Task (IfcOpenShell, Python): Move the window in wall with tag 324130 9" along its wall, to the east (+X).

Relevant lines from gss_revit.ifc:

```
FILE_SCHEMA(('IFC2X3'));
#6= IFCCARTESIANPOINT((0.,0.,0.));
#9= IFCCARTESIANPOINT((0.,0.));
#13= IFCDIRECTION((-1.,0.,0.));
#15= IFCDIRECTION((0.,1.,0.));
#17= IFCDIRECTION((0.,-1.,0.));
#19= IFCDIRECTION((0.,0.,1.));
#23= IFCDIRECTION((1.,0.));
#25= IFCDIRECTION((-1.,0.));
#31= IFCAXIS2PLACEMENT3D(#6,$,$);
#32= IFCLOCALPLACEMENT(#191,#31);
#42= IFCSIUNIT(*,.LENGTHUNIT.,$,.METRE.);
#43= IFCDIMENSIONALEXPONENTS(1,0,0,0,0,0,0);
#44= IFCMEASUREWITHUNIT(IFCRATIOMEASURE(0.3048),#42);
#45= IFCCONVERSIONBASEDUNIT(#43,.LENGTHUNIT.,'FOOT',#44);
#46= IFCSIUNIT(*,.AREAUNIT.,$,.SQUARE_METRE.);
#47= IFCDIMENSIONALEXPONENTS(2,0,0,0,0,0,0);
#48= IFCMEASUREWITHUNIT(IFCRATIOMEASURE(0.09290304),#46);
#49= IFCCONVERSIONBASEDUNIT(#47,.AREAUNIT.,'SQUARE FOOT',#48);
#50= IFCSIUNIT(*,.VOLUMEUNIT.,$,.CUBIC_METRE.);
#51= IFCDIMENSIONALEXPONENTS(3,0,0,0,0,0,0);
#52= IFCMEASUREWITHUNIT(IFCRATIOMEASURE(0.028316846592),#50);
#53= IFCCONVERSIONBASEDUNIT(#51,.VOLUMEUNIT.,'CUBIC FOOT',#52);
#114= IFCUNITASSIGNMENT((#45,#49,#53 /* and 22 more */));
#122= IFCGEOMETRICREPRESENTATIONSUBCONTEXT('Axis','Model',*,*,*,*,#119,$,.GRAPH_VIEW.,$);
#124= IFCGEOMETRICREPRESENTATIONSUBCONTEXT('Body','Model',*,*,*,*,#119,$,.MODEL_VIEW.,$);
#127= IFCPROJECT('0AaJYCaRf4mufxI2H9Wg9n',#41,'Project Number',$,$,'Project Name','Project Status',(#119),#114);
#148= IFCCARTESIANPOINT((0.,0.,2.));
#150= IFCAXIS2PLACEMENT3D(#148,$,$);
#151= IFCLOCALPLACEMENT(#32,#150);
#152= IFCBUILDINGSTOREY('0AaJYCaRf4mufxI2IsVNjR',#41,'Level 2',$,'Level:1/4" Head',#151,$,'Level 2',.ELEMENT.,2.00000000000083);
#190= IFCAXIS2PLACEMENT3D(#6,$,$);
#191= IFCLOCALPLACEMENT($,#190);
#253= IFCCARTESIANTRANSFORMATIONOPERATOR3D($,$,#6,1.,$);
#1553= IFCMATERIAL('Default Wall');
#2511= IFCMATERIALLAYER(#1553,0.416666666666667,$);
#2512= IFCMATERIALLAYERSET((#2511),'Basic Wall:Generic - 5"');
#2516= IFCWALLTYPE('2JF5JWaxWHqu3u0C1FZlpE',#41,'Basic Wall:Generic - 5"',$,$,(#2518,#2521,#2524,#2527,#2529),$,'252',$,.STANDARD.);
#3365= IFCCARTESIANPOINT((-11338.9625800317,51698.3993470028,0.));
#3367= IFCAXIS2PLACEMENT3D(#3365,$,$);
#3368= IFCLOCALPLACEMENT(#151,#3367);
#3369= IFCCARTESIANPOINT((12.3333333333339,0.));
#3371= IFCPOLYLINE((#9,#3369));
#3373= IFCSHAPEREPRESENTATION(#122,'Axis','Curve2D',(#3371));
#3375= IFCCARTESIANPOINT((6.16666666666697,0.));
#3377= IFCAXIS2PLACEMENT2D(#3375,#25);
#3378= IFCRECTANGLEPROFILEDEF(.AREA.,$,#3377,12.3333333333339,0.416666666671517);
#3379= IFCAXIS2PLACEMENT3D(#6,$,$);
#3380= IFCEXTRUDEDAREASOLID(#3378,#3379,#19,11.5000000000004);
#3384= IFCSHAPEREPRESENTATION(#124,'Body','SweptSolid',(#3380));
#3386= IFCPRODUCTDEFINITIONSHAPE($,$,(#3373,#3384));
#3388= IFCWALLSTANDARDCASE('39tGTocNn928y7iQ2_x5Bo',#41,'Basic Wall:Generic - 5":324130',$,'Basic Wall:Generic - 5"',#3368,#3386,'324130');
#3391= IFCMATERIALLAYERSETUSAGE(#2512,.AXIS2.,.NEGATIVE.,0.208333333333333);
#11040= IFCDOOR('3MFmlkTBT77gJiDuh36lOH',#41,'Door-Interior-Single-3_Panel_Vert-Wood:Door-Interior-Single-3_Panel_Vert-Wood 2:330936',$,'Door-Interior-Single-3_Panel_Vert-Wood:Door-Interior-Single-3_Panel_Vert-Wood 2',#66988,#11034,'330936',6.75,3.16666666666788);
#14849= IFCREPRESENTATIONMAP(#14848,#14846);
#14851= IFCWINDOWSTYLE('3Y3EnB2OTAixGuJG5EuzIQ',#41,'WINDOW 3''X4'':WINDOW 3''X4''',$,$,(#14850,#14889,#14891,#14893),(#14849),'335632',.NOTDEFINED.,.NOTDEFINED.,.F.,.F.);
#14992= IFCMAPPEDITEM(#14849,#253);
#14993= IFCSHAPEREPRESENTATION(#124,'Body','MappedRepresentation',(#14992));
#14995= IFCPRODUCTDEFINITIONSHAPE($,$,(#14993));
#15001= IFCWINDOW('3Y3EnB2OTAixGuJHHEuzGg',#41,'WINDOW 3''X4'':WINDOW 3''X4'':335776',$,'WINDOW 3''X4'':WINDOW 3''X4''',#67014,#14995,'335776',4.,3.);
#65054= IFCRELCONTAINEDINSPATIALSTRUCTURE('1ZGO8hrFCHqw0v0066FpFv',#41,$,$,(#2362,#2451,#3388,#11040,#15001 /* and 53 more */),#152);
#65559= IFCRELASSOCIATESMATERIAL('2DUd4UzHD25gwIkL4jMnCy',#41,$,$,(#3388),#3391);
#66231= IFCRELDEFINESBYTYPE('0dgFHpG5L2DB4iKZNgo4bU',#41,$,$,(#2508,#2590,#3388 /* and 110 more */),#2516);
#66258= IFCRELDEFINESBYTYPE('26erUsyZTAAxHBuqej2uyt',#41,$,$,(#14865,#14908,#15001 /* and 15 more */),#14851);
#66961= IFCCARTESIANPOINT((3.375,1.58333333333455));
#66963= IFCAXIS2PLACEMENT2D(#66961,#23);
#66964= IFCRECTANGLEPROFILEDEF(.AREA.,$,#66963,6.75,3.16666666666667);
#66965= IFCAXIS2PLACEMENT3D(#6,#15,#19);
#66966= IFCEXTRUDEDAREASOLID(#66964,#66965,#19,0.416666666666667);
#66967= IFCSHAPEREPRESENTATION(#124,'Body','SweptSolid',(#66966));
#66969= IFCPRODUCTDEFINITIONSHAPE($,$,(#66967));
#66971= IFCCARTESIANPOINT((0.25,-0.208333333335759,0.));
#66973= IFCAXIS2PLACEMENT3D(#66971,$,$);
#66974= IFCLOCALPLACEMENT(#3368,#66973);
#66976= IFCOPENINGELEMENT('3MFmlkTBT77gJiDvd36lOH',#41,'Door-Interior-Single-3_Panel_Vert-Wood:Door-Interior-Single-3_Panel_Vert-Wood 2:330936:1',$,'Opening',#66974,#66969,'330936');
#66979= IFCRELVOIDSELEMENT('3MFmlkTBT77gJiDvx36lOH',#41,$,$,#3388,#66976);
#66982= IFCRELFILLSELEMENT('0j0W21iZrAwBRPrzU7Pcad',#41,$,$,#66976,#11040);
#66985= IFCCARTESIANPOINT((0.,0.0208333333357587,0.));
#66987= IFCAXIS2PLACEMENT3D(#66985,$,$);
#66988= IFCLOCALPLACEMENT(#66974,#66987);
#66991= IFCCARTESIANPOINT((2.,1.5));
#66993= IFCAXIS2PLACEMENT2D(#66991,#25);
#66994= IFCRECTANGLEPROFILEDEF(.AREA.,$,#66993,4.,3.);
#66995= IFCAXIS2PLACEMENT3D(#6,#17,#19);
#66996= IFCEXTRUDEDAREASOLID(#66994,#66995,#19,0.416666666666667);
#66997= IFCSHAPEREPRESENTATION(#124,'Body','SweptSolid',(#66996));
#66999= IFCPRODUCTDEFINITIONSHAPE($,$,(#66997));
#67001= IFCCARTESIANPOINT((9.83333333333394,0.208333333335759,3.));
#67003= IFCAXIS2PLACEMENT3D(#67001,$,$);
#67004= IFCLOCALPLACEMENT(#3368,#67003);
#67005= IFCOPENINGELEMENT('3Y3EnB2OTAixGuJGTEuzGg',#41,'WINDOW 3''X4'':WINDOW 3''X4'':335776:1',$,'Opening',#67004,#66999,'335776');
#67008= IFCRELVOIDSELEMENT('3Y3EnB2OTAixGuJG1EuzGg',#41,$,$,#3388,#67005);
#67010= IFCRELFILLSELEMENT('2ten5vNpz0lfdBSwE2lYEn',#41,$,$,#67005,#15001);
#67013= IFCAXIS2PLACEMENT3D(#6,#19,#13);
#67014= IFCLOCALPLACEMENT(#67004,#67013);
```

```python
import ifcopenshell
import ifcopenshell.api.geometry
import ifcopenshell.util.placement
import ifcopenshell.util.unit

model = ifcopenshell.open("gss_revit.ifc")
unit_scale = ifcopenshell.util.unit.calculate_unit_scale(model)

window = model.by_guid("3Y3EnB2OTAixGuJHHEuzGg")
opening = window.FillsVoids[0].RelatingOpeningElement
wall = opening.VoidsElements[0].RelatingBuildingElement

wall_matrix = ifcopenshell.util.placement.get_local_placement(wall.ObjectPlacement)
shift = wall_matrix[:3, 0] * 9 * 0.0254 / unit_scale
before = ifcopenshell.util.placement.get_local_placement(window.ObjectPlacement)[:3, 3].copy()

# The window is placed relative to its opening, so it follows when the opening moves.
matrix = ifcopenshell.util.placement.get_local_placement(opening.ObjectPlacement)
matrix[:3, 3] += shift
ifcopenshell.api.geometry.edit_object_placement(
    model, product=opening, matrix=matrix, is_si=False, should_transform_children=True
)

after = ifcopenshell.util.placement.get_local_placement(window.ObjectPlacement)[:3, 3]
print("window moved by", (after - before).round(3) + 0.0)

model.write("gss_revit_updated.ifc")
```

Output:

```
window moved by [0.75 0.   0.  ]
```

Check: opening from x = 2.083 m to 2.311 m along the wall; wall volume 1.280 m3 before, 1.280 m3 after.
